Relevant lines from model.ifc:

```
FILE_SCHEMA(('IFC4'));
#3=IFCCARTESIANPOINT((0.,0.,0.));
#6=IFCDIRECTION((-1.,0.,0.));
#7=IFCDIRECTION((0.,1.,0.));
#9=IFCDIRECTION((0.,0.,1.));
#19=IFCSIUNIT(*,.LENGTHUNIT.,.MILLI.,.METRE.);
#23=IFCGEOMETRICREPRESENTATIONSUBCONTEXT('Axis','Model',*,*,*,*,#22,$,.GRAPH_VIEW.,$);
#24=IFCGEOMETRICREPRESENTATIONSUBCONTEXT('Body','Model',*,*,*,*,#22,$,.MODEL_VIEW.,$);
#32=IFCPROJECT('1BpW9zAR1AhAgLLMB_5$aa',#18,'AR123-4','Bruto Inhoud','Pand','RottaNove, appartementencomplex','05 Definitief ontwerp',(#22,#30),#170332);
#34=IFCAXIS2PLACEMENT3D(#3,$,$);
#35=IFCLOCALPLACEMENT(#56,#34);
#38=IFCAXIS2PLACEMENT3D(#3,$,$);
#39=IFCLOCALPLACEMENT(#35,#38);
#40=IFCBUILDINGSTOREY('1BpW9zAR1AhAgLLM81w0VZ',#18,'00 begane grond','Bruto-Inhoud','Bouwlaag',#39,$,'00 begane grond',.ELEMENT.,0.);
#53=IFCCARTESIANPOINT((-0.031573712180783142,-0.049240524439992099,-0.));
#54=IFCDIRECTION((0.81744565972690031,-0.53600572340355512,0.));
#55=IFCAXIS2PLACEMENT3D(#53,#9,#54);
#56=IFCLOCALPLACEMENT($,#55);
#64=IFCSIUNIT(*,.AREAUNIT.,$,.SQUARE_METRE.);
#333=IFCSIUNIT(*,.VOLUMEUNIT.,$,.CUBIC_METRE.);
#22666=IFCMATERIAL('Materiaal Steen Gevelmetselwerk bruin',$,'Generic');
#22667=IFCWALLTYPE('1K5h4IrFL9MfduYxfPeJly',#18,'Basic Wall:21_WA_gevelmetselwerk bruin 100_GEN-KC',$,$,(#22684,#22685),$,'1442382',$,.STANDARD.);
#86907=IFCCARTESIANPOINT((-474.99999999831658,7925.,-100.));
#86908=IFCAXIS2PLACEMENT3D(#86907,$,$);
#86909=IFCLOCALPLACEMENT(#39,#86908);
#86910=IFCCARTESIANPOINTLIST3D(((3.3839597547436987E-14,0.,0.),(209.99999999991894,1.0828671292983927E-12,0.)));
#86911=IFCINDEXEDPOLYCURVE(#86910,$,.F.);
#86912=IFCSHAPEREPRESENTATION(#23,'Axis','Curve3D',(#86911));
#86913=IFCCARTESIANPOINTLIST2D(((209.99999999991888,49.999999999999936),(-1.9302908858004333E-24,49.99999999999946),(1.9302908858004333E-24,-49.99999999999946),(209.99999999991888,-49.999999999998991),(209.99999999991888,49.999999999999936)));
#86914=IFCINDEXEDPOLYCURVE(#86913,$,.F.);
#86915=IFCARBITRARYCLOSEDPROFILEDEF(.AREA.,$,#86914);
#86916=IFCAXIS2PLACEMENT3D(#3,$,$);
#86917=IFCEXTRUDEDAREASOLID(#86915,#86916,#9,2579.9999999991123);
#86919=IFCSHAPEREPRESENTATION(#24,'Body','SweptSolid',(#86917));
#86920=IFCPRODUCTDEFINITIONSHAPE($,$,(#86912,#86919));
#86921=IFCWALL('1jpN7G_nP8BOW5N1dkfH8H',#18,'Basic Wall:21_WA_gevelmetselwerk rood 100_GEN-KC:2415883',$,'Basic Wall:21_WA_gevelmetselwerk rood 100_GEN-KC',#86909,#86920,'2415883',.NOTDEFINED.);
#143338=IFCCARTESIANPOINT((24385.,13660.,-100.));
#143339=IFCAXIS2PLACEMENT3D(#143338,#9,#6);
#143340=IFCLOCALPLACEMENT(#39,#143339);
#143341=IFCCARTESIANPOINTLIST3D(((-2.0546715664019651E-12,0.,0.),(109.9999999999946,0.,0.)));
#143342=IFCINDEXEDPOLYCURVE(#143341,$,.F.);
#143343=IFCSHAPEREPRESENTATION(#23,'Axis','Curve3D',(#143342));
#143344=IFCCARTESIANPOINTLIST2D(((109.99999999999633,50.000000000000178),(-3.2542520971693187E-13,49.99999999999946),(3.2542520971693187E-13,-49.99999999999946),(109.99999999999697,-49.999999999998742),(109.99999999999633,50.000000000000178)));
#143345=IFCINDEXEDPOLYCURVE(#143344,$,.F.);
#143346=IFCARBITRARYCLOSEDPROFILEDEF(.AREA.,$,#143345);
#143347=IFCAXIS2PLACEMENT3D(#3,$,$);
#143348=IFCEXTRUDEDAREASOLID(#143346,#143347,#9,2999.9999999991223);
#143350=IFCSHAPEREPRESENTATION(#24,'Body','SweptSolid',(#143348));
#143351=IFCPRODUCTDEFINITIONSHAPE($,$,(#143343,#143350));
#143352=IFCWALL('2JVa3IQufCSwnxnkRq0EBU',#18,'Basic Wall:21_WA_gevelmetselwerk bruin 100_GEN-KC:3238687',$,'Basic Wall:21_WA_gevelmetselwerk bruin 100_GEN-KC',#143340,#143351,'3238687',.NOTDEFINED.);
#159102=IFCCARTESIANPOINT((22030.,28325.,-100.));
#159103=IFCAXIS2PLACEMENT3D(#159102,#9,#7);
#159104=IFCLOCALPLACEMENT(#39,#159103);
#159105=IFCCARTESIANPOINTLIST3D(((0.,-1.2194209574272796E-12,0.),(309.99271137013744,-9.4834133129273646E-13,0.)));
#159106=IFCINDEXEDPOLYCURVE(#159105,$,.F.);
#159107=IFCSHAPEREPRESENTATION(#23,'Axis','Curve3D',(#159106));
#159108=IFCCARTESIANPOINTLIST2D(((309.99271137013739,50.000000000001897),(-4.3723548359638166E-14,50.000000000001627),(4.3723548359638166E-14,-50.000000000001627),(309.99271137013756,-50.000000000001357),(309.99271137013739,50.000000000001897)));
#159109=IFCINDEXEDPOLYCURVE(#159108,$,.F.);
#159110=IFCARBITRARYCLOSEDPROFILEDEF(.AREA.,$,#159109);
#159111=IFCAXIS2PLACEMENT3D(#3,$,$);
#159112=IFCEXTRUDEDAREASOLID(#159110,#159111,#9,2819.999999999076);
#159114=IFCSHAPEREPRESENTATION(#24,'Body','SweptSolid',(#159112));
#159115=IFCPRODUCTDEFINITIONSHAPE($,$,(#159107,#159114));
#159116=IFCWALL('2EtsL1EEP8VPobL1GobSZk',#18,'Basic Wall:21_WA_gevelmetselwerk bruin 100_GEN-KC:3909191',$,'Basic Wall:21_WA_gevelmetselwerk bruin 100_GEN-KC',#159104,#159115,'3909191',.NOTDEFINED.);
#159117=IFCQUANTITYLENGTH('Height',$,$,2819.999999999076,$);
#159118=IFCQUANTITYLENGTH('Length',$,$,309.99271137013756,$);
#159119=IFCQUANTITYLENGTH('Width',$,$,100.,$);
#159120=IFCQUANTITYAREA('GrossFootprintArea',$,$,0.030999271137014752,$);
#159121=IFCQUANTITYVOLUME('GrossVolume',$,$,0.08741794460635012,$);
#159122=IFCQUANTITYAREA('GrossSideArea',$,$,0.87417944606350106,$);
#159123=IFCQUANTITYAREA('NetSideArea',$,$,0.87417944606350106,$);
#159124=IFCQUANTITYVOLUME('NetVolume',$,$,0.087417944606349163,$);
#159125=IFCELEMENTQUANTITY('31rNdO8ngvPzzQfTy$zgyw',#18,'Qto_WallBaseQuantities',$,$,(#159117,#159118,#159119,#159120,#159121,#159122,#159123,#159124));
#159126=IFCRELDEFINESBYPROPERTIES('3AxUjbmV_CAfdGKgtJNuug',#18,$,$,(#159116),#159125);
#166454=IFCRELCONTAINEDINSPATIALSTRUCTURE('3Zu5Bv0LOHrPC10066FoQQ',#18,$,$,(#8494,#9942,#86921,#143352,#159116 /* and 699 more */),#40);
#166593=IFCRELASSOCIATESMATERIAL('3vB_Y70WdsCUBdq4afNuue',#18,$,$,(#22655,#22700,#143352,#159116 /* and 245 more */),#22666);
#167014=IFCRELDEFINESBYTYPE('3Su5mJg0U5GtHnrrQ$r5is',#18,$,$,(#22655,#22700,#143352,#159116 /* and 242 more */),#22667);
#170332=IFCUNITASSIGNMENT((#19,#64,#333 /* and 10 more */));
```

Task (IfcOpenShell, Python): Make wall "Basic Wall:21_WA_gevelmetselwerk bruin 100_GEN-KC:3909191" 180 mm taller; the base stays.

```python
import ifcopenshell
import ifcopenshell.api.pset
import ifcopenshell.geom
import ifcopenshell.util.element
import ifcopenshell.util.representation
import ifcopenshell.util.shape
import ifcopenshell.util.unit

model = ifcopenshell.open("model.ifc")
unit_scale = ifcopenshell.util.unit.calculate_unit_scale(model)
area_scale = ifcopenshell.util.unit.calculate_unit_scale(model, "AREAUNIT")
volume_scale = ifcopenshell.util.unit.calculate_unit_scale(model, "VOLUMEUNIT")
settings = ifcopenshell.geom.settings()


def volume(element):
    """Net volume in cubic metres, openings subtracted."""
    shape = ifcopenshell.geom.create_shape(settings, element)
    return ifcopenshell.util.shape.get_volume(shape.geometry)


wall = model.by_guid("2EtsL1EEP8VPobL1GobSZk")
before = volume(wall)

body = ifcopenshell.util.representation.get_representation(wall, "Model", "Body")
solid = body.Items[0]
old_height = solid.Depth
solid.Depth += 0.18 / unit_scale
after = volume(wall)
thickness = 0.1  # wall thickness in metres

# Update the stored height, areas and volumes.
qto = model.by_id(ifcopenshell.util.element.get_pset(wall, "Qto_WallBaseQuantities", should_inherit=False)["id"])
ifcopenshell.api.pset.edit_qto(model, qto=qto, properties={
    "Height": solid.Depth,
    "GrossVolume": ifcopenshell.util.element.get_pset(wall, "Qto_WallBaseQuantities", "GrossVolume") * solid.Depth / old_height,
    "GrossSideArea": ifcopenshell.util.element.get_pset(wall, "Qto_WallBaseQuantities", "GrossSideArea") * solid.Depth / old_height,
    "NetSideArea": after / thickness / area_scale,
    "NetVolume": after / volume_scale,
})

print(f"height {old_height:g} -> {solid.Depth:g}, volume {before:.3f} -> {after:.3f} m3")

model.write("model_v2.ifc")
```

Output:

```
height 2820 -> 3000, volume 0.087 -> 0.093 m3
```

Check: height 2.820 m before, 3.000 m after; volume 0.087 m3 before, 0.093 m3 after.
